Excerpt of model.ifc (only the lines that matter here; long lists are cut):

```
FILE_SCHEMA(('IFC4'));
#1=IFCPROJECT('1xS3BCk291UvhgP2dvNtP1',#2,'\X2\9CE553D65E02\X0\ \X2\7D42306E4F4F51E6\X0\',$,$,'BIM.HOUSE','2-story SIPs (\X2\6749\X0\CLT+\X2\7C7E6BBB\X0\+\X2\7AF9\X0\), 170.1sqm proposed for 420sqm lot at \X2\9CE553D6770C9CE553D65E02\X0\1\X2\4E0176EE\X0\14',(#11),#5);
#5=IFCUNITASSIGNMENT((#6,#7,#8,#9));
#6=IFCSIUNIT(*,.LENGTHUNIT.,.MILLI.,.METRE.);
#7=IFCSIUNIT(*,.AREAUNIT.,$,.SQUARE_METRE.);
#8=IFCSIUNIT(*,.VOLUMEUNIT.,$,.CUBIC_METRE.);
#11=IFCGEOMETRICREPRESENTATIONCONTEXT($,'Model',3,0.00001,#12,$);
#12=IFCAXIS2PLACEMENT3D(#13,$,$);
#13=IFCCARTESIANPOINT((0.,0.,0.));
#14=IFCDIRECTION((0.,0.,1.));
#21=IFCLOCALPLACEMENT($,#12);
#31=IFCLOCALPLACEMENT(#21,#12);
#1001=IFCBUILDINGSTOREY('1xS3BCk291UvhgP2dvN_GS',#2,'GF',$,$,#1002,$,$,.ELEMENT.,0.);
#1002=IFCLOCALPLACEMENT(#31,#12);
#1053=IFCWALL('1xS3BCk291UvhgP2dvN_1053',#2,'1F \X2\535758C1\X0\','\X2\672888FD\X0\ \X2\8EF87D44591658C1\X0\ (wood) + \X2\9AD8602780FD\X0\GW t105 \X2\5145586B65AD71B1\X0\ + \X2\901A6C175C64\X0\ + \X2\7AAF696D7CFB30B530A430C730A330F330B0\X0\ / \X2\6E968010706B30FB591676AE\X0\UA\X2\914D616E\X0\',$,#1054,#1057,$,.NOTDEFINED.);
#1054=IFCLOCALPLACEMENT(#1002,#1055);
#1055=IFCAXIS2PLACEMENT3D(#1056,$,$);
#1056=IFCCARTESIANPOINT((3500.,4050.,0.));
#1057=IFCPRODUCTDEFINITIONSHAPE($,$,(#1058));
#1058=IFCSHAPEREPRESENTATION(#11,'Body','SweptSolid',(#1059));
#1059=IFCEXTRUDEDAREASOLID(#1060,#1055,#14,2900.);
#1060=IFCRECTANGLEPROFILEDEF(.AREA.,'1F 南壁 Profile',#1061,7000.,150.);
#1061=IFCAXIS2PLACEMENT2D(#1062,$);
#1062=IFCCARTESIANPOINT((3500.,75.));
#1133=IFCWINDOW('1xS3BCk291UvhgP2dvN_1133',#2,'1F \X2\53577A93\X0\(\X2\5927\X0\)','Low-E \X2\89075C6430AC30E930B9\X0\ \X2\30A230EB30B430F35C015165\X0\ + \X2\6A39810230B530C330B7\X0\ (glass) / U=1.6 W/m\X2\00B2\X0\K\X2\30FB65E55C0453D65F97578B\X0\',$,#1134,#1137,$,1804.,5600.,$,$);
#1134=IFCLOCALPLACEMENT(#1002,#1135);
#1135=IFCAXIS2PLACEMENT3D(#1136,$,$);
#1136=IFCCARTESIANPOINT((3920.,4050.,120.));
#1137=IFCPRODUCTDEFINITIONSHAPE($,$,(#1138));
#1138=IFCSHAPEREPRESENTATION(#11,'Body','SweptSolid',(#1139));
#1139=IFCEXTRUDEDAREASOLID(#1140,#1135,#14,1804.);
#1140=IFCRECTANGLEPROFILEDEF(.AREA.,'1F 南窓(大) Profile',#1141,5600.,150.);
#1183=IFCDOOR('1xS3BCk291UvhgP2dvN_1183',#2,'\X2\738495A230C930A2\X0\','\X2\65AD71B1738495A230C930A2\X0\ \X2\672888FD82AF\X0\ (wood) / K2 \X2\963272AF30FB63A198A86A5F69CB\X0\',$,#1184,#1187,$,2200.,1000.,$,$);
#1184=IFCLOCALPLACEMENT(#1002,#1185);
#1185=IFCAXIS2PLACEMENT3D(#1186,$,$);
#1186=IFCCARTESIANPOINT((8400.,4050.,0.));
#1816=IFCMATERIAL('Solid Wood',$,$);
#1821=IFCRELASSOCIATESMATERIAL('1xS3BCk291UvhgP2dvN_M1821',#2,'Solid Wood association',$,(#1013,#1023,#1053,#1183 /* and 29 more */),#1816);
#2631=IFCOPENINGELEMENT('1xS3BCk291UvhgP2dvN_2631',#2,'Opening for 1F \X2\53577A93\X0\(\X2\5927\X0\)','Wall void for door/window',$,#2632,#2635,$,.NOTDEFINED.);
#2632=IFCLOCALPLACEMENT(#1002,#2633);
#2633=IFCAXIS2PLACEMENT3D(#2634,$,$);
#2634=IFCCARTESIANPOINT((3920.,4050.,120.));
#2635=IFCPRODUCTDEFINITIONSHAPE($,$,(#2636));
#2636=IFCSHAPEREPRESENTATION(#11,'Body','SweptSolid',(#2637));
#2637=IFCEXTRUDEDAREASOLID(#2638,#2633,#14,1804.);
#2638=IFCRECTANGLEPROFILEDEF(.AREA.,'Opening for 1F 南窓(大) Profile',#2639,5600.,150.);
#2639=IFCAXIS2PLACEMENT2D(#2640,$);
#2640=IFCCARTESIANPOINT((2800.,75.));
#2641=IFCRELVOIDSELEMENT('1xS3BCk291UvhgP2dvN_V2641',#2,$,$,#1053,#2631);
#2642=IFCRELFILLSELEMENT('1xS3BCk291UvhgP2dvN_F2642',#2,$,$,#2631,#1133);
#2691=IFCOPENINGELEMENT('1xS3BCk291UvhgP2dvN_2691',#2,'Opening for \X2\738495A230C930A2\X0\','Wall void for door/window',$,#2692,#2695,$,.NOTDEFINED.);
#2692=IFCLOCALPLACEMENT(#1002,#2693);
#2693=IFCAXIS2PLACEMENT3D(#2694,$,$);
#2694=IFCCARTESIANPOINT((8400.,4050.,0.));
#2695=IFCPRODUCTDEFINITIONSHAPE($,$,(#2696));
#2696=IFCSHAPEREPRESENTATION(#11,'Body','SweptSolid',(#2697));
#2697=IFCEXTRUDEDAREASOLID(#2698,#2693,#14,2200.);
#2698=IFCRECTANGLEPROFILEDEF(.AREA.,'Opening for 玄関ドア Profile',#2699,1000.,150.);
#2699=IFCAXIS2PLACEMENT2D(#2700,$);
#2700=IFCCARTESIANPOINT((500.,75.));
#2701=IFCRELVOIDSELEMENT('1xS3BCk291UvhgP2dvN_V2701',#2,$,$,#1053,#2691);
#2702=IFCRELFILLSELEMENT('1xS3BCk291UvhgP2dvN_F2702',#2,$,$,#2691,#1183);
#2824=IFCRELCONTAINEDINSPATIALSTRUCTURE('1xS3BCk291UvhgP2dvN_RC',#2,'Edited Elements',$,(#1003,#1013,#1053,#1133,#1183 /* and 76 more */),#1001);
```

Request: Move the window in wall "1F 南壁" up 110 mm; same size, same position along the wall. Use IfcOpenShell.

```python
import numpy as np
import ifcopenshell
import ifcopenshell.api.geometry
import ifcopenshell.util.placement
import ifcopenshell.util.unit

model = ifcopenshell.open("model.ifc")
unit_scale = ifcopenshell.util.unit.calculate_unit_scale(model)

window = model.by_guid("1xS3BCk291UvhgP2dvN_1133")
opening = window.FillsVoids[0].RelatingOpeningElement
dz = 110.0

shift = np.array([0.0, 0.0, dz])
# The window is not placed relative to its opening, so move both.
for product in (opening, window):
    matrix = ifcopenshell.util.placement.get_local_placement(product.ObjectPlacement)
    matrix[:3, 3] += shift
    ifcopenshell.api.geometry.edit_object_placement(model, product=product, matrix=matrix, is_si=False)

print(f"moved by {dz * unit_scale:+.3f} m")

model.write("model_updated.ifc")
```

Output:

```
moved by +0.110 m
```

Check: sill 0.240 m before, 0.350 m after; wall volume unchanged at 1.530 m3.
